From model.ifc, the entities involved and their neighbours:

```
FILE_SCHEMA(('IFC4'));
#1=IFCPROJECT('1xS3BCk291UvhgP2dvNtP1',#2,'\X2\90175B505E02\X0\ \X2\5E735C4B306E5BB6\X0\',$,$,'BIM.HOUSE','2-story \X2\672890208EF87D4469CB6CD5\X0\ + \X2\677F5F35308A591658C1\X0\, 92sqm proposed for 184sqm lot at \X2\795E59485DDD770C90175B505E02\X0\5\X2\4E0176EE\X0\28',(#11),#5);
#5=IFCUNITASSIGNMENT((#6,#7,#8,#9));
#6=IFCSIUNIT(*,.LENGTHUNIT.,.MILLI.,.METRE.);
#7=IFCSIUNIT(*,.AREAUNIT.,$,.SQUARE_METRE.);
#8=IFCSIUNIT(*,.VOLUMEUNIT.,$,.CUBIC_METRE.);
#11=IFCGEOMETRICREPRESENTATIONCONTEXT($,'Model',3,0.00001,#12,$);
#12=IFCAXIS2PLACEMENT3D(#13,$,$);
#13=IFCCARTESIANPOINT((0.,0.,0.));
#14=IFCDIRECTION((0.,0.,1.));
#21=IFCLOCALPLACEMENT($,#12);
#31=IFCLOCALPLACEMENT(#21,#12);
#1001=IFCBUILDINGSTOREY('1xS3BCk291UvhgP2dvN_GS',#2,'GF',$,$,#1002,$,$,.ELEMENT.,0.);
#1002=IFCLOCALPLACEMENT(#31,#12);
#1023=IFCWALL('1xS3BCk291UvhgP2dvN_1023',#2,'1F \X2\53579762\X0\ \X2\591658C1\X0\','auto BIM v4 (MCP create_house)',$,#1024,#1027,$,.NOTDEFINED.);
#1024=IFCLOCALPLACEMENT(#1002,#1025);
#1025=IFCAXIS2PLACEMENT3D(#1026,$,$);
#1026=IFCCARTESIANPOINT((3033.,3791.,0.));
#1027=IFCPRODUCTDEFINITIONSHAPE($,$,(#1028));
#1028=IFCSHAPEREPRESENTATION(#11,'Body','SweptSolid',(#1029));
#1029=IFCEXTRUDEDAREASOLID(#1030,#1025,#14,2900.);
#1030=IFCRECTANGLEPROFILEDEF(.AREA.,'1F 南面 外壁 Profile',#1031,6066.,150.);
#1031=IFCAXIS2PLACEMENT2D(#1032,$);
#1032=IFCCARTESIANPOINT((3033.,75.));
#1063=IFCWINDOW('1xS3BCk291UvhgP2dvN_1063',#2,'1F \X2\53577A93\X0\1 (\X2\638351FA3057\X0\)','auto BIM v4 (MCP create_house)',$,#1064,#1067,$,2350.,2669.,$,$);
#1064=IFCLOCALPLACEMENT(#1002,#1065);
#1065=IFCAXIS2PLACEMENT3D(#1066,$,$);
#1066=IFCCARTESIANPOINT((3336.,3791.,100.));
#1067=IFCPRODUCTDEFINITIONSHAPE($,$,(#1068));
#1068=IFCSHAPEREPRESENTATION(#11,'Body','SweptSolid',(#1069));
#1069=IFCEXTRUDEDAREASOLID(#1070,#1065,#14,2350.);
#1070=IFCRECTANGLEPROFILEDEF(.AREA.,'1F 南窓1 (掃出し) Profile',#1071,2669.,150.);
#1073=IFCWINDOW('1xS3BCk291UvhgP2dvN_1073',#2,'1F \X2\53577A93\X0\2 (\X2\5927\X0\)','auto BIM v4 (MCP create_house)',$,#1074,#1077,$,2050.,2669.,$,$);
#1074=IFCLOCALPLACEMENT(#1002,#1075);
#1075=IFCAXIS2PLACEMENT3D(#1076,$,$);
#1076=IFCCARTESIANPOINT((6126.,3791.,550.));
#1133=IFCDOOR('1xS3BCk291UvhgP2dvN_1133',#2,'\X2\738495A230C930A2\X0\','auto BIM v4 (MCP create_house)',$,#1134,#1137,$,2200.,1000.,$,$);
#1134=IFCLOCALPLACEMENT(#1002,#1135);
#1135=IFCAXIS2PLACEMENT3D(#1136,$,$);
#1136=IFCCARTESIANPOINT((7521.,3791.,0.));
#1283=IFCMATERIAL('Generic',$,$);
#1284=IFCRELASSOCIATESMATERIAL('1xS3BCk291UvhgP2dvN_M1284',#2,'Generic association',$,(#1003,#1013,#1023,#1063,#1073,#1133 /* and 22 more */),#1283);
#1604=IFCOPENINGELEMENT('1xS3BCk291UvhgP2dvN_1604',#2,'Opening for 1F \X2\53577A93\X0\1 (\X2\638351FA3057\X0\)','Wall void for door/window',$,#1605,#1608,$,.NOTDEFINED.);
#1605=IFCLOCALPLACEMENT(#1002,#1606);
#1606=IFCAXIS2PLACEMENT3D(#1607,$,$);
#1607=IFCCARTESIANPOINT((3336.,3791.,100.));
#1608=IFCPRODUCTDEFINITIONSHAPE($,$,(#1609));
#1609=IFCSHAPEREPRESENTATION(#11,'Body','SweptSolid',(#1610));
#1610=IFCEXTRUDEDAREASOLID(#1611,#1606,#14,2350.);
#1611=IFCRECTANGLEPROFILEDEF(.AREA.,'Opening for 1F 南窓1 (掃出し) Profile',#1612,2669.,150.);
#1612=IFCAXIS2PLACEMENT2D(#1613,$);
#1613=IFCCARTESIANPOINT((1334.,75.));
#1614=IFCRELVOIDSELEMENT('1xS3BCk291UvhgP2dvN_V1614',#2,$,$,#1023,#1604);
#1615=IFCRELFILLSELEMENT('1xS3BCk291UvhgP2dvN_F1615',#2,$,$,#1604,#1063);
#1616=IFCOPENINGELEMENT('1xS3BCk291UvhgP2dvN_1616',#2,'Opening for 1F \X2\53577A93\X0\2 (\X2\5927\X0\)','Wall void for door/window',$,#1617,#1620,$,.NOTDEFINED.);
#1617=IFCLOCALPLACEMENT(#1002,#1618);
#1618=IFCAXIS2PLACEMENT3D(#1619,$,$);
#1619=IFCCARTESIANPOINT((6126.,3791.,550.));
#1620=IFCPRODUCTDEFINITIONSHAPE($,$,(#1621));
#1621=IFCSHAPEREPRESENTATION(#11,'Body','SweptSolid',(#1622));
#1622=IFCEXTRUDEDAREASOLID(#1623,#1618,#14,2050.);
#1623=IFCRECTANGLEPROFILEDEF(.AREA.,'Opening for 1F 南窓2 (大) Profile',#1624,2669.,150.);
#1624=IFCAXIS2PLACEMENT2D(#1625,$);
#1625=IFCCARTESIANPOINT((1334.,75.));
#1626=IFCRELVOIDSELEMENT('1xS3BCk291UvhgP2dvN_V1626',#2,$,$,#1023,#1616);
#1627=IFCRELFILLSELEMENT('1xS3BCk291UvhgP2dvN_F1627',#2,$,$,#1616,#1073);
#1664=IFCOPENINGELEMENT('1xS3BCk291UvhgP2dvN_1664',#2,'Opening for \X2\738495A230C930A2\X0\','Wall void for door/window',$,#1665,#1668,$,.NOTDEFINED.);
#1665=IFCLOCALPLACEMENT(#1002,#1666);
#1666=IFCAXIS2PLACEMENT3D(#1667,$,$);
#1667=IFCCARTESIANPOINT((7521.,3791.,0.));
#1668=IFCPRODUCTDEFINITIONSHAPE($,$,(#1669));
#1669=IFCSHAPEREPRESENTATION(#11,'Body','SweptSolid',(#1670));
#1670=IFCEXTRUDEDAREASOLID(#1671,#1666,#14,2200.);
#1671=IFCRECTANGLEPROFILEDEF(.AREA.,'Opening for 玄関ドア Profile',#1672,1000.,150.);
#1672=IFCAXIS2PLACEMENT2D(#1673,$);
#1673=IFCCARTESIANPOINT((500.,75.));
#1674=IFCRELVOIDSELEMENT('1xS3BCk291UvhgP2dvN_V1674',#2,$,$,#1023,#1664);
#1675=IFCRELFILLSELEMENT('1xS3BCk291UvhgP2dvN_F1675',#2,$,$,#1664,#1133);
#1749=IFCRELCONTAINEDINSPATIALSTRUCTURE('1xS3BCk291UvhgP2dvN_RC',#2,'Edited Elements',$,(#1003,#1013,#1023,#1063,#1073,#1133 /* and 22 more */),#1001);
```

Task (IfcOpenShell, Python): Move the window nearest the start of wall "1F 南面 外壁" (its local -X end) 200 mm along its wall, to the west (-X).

```python
import ifcopenshell
import ifcopenshell.api.geometry
import ifcopenshell.util.placement
import ifcopenshell.util.unit

model = ifcopenshell.open("model.ifc")
unit_scale = ifcopenshell.util.unit.calculate_unit_scale(model)

window = model.by_guid("1xS3BCk291UvhgP2dvN_1063")
opening = window.FillsVoids[0].RelatingOpeningElement
wall = opening.VoidsElements[0].RelatingBuildingElement

wall_matrix = ifcopenshell.util.placement.get_local_placement(wall.ObjectPlacement)
shift = wall_matrix[:3, 0] * -0.2 / unit_scale
before = ifcopenshell.util.placement.get_local_placement(window.ObjectPlacement)[:3, 3].copy()

# The window is not placed relative to its opening, so move both.
for product in (opening, window):
    matrix = ifcopenshell.util.placement.get_local_placement(product.ObjectPlacement)
    matrix[:3, 3] += shift
    ifcopenshell.api.geometry.edit_object_placement(model, product=product, matrix=matrix, is_si=False)

after = ifcopenshell.util.placement.get_local_placement(window.ObjectPlacement)[:3, 3]
print("window moved by", (after - before).round(3) + 0.0)

model.write("model_edited.ifc")
```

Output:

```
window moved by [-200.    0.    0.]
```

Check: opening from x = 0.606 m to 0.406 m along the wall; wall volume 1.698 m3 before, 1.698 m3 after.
